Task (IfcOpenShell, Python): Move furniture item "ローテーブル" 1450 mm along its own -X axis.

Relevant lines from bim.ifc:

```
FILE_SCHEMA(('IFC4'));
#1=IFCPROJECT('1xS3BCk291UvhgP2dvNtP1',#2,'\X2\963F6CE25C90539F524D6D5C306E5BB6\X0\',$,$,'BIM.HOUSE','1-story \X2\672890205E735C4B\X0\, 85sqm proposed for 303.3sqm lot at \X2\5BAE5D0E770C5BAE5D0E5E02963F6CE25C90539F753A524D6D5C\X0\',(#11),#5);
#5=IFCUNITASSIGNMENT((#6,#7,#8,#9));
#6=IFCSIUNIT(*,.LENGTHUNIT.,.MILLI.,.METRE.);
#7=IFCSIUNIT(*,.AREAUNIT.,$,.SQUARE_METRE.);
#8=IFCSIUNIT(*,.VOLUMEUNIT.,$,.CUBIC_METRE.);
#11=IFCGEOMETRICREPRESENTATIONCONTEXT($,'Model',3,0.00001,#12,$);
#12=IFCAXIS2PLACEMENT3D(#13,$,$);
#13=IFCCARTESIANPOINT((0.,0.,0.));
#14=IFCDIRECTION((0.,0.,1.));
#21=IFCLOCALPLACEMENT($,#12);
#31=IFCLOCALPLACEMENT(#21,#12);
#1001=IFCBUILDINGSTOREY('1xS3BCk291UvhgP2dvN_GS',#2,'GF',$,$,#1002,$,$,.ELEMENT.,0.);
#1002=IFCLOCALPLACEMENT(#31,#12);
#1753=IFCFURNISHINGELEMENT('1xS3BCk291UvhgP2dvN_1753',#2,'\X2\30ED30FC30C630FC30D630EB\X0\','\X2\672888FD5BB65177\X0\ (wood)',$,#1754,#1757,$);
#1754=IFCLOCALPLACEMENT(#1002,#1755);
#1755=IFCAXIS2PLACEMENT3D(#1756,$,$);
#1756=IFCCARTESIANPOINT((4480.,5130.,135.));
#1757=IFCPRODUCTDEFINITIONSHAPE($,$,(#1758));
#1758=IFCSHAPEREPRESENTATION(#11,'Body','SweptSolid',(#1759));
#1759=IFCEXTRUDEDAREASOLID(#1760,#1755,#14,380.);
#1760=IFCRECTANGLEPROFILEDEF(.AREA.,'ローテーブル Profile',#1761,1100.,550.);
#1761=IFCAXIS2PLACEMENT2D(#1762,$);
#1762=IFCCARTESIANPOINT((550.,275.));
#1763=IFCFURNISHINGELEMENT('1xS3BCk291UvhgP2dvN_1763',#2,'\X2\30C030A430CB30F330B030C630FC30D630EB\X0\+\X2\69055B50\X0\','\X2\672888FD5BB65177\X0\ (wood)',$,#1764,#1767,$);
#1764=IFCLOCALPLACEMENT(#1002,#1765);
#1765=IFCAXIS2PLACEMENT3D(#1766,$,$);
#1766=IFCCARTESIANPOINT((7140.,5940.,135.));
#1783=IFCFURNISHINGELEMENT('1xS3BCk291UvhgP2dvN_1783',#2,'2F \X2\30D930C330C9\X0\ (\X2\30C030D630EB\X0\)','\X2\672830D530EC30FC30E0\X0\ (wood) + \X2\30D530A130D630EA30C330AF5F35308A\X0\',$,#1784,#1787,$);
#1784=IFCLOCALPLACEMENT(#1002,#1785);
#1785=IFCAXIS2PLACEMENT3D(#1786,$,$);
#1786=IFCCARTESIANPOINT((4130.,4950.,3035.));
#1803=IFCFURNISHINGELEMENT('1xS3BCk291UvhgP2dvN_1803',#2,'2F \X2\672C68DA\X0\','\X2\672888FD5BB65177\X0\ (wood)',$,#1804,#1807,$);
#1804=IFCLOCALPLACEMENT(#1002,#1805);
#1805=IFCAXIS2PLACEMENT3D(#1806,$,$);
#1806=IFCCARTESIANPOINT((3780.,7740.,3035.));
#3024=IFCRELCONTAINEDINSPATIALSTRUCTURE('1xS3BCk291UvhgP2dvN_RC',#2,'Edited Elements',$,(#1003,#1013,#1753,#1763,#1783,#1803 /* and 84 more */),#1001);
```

```python
import ifcopenshell
import ifcopenshell.api.geometry
import ifcopenshell.util.placement

model = ifcopenshell.open("bim.ifc")

item = model.by_guid("1xS3BCk291UvhgP2dvN_1753")
matrix = ifcopenshell.util.placement.get_local_placement(item.ObjectPlacement)
matrix[:3, 3] -= matrix[:3, 0] * 1450.0
ifcopenshell.api.geometry.edit_object_placement(model, product=item, matrix=matrix, is_si=False)

print(ifcopenshell.util.placement.get_local_placement(item.ObjectPlacement).round(3) + 0.0)

model.write("bim_edited.ifc")
```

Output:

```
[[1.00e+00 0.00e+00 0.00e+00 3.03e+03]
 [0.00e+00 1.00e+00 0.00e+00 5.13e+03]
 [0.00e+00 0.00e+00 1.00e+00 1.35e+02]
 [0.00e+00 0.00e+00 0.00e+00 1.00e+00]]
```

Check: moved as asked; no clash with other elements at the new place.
